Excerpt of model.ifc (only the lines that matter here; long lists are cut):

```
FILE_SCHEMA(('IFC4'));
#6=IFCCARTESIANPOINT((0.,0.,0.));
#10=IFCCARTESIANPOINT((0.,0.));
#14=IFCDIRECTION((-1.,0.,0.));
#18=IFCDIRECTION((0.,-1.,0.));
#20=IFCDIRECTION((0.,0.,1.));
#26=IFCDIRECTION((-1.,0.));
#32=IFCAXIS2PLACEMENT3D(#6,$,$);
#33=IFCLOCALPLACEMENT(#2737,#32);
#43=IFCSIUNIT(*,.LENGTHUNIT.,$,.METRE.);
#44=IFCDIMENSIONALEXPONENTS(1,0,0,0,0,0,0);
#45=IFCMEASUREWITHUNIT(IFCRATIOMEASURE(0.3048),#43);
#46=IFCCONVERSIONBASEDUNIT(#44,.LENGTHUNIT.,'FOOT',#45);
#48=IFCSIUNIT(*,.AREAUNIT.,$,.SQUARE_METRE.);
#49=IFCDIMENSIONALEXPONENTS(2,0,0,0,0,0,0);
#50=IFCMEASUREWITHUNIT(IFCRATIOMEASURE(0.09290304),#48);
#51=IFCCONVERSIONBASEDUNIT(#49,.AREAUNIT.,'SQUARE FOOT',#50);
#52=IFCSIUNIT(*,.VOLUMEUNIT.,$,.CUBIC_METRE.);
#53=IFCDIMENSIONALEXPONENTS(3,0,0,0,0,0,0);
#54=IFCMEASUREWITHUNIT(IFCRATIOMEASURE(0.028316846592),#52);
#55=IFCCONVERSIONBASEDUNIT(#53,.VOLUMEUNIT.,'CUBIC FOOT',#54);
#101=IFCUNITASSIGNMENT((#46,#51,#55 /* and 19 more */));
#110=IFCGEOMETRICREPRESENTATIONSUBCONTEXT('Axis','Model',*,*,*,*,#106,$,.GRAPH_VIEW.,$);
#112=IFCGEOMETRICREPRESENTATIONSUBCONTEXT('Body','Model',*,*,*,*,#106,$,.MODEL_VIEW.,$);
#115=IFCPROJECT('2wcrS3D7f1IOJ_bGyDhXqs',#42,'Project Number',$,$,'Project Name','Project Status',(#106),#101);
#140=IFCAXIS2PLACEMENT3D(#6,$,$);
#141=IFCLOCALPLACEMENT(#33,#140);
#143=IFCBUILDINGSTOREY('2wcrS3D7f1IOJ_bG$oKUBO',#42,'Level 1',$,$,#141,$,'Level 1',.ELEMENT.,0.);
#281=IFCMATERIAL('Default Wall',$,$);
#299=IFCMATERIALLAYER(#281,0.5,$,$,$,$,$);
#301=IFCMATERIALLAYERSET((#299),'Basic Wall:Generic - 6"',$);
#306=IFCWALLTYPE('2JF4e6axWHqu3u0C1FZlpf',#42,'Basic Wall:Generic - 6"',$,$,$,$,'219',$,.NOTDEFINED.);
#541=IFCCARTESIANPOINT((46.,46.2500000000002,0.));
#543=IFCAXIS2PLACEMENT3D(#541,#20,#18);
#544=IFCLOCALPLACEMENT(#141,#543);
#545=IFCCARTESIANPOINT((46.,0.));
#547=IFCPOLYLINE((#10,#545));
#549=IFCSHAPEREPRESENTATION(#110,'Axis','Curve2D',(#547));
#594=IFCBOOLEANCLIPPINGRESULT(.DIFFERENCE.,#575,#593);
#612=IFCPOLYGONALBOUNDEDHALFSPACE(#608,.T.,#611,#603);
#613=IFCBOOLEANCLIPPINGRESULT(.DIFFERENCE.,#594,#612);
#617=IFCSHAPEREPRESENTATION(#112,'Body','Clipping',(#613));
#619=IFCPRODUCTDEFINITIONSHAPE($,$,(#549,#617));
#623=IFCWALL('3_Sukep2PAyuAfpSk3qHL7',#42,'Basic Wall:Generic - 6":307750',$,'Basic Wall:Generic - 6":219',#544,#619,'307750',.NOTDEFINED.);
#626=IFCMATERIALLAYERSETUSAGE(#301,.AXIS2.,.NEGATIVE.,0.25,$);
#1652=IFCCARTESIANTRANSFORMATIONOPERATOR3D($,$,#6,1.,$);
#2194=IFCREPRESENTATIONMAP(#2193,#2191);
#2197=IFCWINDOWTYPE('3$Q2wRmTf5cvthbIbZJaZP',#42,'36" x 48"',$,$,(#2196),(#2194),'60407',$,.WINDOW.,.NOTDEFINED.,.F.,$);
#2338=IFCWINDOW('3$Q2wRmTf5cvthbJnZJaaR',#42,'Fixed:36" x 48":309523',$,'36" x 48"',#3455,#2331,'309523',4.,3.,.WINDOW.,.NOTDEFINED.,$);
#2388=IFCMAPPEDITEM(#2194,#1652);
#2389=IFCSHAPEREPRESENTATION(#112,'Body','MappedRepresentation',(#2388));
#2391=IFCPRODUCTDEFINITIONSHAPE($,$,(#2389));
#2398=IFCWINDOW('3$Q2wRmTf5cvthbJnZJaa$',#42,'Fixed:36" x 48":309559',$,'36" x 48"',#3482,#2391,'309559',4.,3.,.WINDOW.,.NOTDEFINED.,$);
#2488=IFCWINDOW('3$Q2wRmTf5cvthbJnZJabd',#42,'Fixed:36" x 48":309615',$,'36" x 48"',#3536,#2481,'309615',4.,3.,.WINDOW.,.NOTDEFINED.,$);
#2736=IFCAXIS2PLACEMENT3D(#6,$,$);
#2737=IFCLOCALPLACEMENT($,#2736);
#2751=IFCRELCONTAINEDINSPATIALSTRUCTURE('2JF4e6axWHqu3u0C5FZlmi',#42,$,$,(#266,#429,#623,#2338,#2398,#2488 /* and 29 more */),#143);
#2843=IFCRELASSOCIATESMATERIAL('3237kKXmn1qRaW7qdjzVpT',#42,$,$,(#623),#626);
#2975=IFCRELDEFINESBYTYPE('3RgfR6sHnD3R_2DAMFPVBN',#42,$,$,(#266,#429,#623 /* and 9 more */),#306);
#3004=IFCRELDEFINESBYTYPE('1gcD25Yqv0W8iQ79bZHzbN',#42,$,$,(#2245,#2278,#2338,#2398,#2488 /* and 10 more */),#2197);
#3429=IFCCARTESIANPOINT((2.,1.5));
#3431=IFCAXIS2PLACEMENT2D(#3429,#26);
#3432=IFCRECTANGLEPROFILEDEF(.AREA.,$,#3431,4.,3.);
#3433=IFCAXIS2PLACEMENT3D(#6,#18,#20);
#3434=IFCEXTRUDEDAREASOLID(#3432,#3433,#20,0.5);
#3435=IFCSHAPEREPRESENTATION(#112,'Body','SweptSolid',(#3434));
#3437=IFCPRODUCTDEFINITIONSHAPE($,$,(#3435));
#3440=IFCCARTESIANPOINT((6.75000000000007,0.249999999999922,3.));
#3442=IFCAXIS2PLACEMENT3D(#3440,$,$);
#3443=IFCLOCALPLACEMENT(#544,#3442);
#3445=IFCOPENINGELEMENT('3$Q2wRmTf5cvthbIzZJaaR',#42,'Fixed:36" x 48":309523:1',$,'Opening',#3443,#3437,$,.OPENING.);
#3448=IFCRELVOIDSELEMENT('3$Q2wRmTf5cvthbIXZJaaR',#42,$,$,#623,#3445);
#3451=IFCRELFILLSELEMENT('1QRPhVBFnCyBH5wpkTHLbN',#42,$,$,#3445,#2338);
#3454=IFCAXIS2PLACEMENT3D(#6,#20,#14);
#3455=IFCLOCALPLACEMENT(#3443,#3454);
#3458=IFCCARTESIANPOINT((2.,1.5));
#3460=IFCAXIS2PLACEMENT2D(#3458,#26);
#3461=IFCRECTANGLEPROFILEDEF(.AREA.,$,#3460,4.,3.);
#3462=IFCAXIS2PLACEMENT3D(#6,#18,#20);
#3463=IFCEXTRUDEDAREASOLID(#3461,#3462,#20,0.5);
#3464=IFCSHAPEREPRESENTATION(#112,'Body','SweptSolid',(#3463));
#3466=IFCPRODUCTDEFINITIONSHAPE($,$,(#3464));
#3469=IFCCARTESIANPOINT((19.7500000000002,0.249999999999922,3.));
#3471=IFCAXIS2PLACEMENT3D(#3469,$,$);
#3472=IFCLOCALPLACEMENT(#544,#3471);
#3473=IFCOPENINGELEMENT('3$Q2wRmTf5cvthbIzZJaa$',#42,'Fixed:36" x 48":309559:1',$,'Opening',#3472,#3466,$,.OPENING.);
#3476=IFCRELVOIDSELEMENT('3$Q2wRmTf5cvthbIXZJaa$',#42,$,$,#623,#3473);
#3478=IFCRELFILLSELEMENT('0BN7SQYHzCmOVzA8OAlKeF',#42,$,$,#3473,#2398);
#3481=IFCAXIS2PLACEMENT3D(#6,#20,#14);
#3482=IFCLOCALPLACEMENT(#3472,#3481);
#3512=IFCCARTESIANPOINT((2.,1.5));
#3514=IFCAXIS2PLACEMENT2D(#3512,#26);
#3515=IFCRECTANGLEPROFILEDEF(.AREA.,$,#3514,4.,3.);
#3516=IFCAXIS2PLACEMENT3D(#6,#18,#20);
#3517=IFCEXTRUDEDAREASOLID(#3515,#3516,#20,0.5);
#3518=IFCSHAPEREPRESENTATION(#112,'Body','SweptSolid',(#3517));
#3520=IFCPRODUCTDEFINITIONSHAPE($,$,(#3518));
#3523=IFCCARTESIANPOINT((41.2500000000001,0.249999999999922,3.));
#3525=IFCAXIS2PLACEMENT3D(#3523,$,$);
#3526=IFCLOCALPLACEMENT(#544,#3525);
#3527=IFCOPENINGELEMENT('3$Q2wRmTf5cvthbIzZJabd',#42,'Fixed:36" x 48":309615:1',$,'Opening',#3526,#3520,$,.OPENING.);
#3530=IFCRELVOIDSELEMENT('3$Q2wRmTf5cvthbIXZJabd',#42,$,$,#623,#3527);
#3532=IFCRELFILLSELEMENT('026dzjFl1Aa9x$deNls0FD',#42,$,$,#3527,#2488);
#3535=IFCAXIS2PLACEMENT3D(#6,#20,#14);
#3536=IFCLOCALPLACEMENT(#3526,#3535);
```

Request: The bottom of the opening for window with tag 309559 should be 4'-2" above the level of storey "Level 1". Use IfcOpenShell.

```python
import numpy as np
import ifcopenshell
import ifcopenshell.api.geometry
import ifcopenshell.geom
import ifcopenshell.util.element
import ifcopenshell.util.placement
import ifcopenshell.util.shape
import ifcopenshell.util.unit

model = ifcopenshell.open("model.ifc")
unit_scale = ifcopenshell.util.unit.calculate_unit_scale(model)

window = model.by_guid("3$Q2wRmTf5cvthbJnZJaa$")
opening = window.FillsVoids[0].RelatingOpeningElement
storey = ifcopenshell.util.element.get_container(window, ifc_class="IfcBuildingStorey")
level = ifcopenshell.util.placement.get_local_placement(storey.ObjectPlacement)[2, 3]

# The opening's origin need not be at the sill, so measure its lowest point.
shape = ifcopenshell.geom.create_shape(ifcopenshell.geom.settings(), opening)
bottom = ifcopenshell.util.shape.get_shape_bottom_elevation(shape, shape.geometry) / unit_scale
dz = level + 50 * 0.0254 / unit_scale - bottom

shift = np.array([0.0, 0.0, dz])
# The window is placed relative to its opening, so it follows when the opening moves.
matrix = ifcopenshell.util.placement.get_local_placement(opening.ObjectPlacement)
matrix[:3, 3] += shift
ifcopenshell.api.geometry.edit_object_placement(
    model, product=opening, matrix=matrix, is_si=False, should_transform_children=True
)

print(f"moved by {dz * unit_scale:+.3f} m")

model.write("model_edited.ifc")
```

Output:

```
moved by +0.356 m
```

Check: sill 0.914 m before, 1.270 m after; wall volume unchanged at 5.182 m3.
